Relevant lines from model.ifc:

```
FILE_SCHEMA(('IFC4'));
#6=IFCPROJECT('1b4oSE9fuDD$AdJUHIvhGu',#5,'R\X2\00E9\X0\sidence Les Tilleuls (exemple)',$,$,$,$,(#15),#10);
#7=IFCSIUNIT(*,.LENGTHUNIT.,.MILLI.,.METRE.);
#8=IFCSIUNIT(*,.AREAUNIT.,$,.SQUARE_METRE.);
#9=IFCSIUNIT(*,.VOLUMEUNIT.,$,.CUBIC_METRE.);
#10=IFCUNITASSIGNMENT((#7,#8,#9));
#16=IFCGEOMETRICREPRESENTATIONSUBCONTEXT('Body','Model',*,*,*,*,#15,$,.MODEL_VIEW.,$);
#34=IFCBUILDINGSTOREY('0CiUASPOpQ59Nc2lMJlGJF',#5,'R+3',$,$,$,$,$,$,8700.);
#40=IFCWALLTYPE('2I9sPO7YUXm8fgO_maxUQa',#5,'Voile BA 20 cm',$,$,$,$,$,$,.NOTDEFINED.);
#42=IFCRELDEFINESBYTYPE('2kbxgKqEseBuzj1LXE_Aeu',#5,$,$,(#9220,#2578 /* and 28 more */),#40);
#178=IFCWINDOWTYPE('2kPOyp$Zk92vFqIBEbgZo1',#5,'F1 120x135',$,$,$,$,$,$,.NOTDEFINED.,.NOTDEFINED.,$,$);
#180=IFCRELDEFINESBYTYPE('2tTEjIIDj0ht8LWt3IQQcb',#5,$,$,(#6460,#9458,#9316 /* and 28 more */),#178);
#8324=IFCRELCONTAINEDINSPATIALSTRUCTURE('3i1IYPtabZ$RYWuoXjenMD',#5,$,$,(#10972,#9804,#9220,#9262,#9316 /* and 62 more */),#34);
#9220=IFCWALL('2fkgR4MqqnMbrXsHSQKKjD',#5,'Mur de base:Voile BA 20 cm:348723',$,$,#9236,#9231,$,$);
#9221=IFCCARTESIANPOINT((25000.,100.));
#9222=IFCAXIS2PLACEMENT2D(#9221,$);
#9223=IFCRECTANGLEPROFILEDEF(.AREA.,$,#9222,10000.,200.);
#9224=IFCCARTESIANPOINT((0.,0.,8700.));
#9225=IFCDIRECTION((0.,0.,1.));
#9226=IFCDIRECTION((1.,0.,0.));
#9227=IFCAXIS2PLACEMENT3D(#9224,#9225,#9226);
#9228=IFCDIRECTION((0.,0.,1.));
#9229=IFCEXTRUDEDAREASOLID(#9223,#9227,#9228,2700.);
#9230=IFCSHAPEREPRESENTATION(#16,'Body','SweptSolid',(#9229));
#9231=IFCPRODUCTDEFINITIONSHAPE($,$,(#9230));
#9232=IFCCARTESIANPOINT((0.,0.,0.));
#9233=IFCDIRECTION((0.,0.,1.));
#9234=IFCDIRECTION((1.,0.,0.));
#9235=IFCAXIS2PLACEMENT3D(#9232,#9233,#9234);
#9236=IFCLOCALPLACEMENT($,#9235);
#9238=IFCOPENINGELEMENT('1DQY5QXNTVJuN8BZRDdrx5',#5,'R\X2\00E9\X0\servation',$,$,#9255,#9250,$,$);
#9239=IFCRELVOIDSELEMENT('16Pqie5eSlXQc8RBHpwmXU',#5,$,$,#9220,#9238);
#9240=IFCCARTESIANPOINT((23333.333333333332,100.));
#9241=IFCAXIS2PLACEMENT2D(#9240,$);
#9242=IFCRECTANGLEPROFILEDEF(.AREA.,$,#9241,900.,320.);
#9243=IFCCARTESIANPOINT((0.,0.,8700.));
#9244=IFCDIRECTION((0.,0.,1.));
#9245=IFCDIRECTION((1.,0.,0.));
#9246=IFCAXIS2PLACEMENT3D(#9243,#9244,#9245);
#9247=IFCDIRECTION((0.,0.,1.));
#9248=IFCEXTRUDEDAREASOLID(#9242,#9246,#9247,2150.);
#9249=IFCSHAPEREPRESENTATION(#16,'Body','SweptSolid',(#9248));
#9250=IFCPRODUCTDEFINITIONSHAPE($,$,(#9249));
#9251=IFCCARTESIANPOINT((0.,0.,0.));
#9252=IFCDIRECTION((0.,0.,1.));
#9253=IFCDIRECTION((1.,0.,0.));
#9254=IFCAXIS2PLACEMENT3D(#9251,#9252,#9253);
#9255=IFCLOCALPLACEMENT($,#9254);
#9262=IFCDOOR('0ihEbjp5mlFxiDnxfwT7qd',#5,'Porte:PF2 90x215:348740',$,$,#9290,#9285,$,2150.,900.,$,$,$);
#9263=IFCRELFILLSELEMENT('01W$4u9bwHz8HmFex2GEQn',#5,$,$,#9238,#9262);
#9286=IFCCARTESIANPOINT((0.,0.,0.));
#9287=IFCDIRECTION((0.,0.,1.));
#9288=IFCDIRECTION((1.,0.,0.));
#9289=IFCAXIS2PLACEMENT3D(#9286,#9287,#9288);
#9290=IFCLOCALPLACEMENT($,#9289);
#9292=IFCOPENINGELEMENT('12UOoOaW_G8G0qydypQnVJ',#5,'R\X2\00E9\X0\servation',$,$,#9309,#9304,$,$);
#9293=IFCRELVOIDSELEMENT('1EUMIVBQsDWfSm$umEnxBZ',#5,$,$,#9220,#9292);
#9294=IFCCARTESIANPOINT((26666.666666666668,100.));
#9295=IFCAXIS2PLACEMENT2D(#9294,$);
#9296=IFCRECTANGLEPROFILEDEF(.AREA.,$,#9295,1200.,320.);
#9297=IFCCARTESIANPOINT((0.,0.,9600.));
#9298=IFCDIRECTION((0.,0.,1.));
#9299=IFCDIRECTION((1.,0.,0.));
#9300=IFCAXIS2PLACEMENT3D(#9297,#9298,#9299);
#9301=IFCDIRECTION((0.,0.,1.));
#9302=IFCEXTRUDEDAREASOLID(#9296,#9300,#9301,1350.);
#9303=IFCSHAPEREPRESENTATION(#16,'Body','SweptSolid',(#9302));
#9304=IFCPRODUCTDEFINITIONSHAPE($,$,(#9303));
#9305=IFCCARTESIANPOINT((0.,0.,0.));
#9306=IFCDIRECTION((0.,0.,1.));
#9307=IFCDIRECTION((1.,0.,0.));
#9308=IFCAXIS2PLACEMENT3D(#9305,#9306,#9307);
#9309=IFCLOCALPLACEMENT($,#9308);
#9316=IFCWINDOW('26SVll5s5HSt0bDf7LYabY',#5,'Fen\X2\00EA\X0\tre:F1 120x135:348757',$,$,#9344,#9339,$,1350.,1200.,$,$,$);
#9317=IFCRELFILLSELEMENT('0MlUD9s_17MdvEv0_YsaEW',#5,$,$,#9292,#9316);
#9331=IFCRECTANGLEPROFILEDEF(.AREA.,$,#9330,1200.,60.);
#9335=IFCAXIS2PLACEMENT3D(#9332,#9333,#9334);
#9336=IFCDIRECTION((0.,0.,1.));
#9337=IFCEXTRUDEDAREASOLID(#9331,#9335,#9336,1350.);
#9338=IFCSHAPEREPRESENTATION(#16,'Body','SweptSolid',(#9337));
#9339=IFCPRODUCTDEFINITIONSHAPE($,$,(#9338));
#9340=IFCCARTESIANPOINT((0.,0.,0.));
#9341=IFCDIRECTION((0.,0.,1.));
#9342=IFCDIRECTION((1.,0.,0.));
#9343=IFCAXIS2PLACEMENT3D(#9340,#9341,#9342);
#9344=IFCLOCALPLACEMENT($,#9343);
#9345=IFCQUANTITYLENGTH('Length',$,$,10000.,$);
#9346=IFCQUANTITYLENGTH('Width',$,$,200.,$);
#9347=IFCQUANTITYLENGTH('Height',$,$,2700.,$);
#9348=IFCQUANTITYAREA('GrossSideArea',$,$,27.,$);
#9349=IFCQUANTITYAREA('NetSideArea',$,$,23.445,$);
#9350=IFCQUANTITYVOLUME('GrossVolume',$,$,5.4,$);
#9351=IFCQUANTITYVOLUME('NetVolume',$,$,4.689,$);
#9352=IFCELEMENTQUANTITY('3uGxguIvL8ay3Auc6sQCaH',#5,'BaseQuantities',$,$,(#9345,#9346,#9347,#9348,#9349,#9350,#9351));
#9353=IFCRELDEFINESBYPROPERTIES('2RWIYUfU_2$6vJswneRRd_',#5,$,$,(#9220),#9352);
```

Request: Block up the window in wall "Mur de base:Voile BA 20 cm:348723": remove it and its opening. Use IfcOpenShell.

```python
import ifcopenshell
import ifcopenshell.api.feature
import ifcopenshell.api.pset
import ifcopenshell.api.root
import ifcopenshell.geom
import ifcopenshell.util.element
import ifcopenshell.util.shape
import ifcopenshell.util.unit

model = ifcopenshell.open("model.ifc")
area_scale = ifcopenshell.util.unit.calculate_unit_scale(model, "AREAUNIT")
volume_scale = ifcopenshell.util.unit.calculate_unit_scale(model, "VOLUMEUNIT")
settings = ifcopenshell.geom.settings()


def volume(element):
    """Net volume in cubic metres, openings subtracted."""
    shape = ifcopenshell.geom.create_shape(settings, element)
    return ifcopenshell.util.shape.get_volume(shape.geometry)


window = model.by_guid("26SVll5s5HSt0bDf7LYabY")
opening = window.FillsVoids[0].RelatingOpeningElement
wall = opening.VoidsElements[0].RelatingBuildingElement
before = volume(wall)

ifcopenshell.api.root.remove_product(model, product=window)
ifcopenshell.api.feature.remove_feature(model, feature=opening)

after = volume(wall)
thickness = 0.2  # wall thickness in metres

# Update the wall's stored quantities.
qto = model.by_id(ifcopenshell.util.element.get_pset(wall, "BaseQuantities", should_inherit=False)["id"])
ifcopenshell.api.pset.edit_qto(model, qto=qto, properties={
    "NetSideArea": after / thickness / area_scale,
    "NetVolume": after / volume_scale,
})

print(f"wall volume {before:.3f} -> {after:.3f} m3")

model.write("model-out.ifc")
```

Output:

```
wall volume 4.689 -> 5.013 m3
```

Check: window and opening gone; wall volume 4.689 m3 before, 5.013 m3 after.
